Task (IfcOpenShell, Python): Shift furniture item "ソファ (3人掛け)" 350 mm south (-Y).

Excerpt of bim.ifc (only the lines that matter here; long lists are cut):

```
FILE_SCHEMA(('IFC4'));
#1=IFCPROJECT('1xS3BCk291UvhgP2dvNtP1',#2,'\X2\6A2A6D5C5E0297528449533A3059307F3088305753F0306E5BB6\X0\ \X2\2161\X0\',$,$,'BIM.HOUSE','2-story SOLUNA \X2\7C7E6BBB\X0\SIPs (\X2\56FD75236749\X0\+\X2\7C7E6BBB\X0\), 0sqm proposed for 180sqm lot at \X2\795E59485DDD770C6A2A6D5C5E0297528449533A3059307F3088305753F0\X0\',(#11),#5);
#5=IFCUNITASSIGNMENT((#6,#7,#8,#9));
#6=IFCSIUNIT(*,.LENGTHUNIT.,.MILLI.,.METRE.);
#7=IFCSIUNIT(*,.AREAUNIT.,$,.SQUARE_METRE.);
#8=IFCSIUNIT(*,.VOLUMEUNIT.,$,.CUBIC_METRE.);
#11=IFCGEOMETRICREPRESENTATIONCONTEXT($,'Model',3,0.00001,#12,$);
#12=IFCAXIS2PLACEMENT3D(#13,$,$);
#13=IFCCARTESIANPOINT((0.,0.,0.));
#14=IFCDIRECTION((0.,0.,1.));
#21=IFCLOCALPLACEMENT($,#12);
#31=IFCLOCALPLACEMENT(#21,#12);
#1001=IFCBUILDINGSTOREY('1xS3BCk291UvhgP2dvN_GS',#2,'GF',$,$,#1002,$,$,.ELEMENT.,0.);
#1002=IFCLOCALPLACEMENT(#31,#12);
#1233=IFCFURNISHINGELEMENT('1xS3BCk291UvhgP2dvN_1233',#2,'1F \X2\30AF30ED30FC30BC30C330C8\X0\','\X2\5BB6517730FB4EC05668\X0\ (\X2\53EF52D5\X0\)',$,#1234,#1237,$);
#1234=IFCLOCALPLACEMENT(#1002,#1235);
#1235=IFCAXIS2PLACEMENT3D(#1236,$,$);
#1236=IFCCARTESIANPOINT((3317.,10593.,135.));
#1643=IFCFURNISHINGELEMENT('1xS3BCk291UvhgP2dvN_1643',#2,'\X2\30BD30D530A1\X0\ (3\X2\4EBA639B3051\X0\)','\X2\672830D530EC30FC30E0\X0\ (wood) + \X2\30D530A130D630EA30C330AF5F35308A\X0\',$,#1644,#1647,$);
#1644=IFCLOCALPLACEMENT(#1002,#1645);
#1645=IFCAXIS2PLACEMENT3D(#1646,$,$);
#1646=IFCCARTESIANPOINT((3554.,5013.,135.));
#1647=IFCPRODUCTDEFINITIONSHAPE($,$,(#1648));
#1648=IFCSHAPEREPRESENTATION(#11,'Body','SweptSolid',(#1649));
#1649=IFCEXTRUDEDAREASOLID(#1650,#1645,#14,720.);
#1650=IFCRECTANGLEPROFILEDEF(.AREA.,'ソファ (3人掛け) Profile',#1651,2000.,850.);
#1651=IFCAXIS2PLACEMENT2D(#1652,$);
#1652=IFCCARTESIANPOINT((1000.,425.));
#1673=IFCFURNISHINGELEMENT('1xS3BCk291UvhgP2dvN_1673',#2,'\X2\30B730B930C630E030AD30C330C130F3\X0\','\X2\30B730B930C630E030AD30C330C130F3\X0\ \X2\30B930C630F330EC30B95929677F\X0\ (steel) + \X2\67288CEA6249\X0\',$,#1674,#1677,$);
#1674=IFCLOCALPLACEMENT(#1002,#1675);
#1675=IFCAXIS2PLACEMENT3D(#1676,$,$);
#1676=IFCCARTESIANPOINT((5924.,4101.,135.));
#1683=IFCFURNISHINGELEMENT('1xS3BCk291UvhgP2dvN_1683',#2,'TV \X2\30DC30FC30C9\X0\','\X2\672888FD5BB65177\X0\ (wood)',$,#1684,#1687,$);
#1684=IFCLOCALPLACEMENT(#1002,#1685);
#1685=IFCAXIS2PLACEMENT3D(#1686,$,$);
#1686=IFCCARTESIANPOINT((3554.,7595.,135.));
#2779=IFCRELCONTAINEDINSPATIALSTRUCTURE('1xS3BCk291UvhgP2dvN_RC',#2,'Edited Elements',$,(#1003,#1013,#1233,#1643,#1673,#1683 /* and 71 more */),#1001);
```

```python
import ifcopenshell
import ifcopenshell.api.geometry
import ifcopenshell.util.placement
import ifcopenshell.util.unit

model = ifcopenshell.open("bim.ifc")
unit_scale = ifcopenshell.util.unit.calculate_unit_scale(model)

item = model.by_guid("1xS3BCk291UvhgP2dvN_1643")
matrix = ifcopenshell.util.placement.get_local_placement(item.ObjectPlacement)
matrix[1, 3] -= 0.35 / unit_scale
ifcopenshell.api.geometry.edit_object_placement(model, product=item, matrix=matrix, is_si=False)

print(ifcopenshell.util.placement.get_local_placement(item.ObjectPlacement).round(3) + 0.0)

model.write("bim_edited.ifc")
```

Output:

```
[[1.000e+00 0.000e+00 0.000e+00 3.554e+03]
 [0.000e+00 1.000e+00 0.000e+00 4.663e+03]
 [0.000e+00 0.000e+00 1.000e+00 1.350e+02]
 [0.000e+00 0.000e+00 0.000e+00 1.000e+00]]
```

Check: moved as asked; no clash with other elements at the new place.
